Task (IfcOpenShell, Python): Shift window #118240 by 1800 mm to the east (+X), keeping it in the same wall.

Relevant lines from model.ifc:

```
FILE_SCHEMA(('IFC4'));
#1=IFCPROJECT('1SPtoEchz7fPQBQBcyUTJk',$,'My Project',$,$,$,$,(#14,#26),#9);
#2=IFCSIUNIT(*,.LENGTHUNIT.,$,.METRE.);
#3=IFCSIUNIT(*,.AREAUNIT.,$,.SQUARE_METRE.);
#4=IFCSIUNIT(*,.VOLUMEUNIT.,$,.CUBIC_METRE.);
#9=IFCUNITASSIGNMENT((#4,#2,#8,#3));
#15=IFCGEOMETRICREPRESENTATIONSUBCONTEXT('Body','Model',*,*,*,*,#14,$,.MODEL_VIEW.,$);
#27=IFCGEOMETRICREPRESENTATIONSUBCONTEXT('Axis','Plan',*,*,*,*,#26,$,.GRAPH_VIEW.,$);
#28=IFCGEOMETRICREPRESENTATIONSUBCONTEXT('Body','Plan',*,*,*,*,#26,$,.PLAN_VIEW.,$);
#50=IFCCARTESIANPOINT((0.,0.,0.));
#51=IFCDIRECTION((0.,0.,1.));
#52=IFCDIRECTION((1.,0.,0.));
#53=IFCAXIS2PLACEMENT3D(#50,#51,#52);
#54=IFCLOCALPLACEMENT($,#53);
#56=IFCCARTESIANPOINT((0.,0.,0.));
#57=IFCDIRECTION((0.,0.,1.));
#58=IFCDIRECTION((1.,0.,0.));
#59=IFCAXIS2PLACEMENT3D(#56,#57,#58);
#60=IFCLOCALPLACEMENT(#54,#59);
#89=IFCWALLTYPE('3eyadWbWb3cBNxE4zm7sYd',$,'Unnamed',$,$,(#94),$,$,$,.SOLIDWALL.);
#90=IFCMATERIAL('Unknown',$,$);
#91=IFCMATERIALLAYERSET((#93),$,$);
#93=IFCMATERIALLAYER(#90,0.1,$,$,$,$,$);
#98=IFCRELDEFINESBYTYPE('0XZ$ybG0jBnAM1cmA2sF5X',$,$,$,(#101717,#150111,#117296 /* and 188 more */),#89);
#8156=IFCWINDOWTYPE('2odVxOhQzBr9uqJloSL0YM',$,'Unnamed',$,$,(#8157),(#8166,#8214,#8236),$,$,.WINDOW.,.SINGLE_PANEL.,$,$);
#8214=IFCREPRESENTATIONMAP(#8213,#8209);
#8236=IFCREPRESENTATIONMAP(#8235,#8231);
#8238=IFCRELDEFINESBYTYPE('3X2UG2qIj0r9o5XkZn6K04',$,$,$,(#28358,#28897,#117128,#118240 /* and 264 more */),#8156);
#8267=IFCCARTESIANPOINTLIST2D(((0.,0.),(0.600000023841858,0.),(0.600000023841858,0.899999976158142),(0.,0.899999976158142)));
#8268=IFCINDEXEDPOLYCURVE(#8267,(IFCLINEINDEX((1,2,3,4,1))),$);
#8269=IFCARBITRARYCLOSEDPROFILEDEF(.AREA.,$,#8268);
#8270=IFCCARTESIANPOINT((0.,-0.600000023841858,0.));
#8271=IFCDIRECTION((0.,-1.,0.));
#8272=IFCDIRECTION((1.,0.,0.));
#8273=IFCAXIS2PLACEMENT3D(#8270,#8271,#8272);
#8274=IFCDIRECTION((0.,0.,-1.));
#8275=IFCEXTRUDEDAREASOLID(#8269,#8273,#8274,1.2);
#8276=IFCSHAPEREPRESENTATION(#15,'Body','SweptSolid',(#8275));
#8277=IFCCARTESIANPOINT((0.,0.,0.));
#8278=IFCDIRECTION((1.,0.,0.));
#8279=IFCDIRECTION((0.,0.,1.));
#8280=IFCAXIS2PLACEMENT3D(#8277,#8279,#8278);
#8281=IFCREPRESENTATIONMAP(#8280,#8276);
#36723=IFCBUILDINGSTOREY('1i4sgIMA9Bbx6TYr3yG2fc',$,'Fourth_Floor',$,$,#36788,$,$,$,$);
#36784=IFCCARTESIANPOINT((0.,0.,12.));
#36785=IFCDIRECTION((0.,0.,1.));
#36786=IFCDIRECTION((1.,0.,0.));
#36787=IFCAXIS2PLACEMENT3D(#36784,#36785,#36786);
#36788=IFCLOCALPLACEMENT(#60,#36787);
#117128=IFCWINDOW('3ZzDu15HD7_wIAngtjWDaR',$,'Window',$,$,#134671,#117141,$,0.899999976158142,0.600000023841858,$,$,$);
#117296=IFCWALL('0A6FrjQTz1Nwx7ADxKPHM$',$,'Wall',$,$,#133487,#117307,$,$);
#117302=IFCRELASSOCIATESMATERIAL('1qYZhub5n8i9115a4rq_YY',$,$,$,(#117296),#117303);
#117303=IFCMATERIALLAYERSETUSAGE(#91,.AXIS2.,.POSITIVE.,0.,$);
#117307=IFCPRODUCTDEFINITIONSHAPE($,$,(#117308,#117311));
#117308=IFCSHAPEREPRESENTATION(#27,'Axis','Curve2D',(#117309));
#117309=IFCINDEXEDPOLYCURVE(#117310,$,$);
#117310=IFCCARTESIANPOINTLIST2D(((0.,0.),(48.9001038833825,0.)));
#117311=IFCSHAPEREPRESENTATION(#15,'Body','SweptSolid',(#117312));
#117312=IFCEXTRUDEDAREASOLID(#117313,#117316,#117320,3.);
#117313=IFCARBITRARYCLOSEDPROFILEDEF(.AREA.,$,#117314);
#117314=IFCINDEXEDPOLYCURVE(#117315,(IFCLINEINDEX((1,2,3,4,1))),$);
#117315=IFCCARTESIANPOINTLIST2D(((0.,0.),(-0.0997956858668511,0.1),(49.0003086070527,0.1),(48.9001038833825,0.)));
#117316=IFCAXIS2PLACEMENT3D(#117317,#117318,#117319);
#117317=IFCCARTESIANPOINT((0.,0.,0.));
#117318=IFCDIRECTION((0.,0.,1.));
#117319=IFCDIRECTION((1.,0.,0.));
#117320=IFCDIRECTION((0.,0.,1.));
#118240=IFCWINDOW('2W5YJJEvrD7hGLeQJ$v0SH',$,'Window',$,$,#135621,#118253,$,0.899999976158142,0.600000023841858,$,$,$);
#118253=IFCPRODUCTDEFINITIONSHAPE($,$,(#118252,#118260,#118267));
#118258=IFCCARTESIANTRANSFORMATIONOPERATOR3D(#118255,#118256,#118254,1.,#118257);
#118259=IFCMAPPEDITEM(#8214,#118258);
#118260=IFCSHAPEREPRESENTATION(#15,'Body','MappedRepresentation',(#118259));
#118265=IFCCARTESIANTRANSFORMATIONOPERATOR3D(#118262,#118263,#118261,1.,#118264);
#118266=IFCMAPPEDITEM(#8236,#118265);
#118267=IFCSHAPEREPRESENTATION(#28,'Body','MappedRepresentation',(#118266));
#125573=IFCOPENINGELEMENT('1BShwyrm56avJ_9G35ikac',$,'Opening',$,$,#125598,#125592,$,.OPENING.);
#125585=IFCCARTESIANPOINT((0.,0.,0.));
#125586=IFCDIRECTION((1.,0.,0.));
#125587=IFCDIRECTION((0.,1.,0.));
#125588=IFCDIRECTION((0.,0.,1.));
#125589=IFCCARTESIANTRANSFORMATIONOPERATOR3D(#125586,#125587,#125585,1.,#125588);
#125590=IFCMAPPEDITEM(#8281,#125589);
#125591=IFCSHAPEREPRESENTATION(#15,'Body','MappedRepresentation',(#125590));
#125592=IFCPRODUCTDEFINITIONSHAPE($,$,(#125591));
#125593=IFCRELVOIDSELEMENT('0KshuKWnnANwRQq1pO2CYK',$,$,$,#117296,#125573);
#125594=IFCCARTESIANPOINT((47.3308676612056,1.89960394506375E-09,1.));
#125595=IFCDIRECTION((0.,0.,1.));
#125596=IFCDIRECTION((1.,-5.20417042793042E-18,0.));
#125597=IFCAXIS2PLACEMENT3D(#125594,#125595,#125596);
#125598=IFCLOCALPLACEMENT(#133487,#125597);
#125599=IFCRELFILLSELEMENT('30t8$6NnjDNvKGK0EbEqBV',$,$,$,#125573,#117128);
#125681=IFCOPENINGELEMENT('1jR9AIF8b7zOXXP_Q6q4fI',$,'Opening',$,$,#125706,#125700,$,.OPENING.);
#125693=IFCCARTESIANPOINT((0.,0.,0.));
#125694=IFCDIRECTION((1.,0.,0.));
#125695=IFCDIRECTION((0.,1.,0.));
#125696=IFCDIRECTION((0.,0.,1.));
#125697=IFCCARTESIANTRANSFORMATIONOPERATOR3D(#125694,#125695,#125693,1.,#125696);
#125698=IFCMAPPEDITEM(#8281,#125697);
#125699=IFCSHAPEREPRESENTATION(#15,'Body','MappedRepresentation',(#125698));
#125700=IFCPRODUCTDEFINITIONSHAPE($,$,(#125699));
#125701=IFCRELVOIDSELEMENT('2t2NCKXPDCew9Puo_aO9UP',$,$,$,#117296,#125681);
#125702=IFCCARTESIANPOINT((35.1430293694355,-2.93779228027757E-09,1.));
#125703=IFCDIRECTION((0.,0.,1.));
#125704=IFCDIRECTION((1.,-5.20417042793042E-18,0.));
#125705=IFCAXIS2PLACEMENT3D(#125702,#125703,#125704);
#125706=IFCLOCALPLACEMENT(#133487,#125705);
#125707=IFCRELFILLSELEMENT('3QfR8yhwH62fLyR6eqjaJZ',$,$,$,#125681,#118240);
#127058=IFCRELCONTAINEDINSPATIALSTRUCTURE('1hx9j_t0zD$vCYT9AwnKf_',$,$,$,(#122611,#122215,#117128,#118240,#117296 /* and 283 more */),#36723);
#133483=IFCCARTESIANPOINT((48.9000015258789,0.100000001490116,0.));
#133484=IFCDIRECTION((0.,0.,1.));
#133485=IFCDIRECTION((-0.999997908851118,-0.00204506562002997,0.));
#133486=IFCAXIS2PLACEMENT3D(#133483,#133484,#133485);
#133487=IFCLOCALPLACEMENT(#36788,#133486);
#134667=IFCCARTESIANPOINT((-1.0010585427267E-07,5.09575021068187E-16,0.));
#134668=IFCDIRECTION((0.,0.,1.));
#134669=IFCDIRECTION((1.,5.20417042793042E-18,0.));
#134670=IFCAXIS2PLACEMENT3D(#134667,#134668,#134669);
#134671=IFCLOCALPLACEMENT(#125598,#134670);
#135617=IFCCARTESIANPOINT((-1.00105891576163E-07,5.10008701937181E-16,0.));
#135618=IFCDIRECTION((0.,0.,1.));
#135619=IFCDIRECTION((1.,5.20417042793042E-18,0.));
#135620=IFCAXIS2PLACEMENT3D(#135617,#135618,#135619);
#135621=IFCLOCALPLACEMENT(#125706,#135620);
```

```python
import ifcopenshell
import ifcopenshell.api.geometry
import ifcopenshell.util.placement

model = ifcopenshell.open("model.ifc")

window = model.by_guid("2W5YJJEvrD7hGLeQJ$v0SH")
opening = window.FillsVoids[0].RelatingOpeningElement
wall = opening.VoidsElements[0].RelatingBuildingElement

wall_matrix = ifcopenshell.util.placement.get_local_placement(wall.ObjectPlacement)
shift = wall_matrix[:3, 0] * -1.8
before = ifcopenshell.util.placement.get_local_placement(window.ObjectPlacement)[:3, 3].copy()

# The window is placed relative to its opening, so it follows when the opening moves.
matrix = ifcopenshell.util.placement.get_local_placement(opening.ObjectPlacement)
matrix[:3, 3] += shift
ifcopenshell.api.geometry.edit_object_placement(
    model, product=opening, matrix=matrix, is_si=False, should_transform_children=True
)

after = ifcopenshell.util.placement.get_local_placement(window.ObjectPlacement)[:3, 3]
print("window moved by", (after - before).round(3) + 0.0)

model.write("model_updated.ifc")
```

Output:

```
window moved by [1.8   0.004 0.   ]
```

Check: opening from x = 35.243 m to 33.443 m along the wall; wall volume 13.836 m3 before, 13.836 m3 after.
